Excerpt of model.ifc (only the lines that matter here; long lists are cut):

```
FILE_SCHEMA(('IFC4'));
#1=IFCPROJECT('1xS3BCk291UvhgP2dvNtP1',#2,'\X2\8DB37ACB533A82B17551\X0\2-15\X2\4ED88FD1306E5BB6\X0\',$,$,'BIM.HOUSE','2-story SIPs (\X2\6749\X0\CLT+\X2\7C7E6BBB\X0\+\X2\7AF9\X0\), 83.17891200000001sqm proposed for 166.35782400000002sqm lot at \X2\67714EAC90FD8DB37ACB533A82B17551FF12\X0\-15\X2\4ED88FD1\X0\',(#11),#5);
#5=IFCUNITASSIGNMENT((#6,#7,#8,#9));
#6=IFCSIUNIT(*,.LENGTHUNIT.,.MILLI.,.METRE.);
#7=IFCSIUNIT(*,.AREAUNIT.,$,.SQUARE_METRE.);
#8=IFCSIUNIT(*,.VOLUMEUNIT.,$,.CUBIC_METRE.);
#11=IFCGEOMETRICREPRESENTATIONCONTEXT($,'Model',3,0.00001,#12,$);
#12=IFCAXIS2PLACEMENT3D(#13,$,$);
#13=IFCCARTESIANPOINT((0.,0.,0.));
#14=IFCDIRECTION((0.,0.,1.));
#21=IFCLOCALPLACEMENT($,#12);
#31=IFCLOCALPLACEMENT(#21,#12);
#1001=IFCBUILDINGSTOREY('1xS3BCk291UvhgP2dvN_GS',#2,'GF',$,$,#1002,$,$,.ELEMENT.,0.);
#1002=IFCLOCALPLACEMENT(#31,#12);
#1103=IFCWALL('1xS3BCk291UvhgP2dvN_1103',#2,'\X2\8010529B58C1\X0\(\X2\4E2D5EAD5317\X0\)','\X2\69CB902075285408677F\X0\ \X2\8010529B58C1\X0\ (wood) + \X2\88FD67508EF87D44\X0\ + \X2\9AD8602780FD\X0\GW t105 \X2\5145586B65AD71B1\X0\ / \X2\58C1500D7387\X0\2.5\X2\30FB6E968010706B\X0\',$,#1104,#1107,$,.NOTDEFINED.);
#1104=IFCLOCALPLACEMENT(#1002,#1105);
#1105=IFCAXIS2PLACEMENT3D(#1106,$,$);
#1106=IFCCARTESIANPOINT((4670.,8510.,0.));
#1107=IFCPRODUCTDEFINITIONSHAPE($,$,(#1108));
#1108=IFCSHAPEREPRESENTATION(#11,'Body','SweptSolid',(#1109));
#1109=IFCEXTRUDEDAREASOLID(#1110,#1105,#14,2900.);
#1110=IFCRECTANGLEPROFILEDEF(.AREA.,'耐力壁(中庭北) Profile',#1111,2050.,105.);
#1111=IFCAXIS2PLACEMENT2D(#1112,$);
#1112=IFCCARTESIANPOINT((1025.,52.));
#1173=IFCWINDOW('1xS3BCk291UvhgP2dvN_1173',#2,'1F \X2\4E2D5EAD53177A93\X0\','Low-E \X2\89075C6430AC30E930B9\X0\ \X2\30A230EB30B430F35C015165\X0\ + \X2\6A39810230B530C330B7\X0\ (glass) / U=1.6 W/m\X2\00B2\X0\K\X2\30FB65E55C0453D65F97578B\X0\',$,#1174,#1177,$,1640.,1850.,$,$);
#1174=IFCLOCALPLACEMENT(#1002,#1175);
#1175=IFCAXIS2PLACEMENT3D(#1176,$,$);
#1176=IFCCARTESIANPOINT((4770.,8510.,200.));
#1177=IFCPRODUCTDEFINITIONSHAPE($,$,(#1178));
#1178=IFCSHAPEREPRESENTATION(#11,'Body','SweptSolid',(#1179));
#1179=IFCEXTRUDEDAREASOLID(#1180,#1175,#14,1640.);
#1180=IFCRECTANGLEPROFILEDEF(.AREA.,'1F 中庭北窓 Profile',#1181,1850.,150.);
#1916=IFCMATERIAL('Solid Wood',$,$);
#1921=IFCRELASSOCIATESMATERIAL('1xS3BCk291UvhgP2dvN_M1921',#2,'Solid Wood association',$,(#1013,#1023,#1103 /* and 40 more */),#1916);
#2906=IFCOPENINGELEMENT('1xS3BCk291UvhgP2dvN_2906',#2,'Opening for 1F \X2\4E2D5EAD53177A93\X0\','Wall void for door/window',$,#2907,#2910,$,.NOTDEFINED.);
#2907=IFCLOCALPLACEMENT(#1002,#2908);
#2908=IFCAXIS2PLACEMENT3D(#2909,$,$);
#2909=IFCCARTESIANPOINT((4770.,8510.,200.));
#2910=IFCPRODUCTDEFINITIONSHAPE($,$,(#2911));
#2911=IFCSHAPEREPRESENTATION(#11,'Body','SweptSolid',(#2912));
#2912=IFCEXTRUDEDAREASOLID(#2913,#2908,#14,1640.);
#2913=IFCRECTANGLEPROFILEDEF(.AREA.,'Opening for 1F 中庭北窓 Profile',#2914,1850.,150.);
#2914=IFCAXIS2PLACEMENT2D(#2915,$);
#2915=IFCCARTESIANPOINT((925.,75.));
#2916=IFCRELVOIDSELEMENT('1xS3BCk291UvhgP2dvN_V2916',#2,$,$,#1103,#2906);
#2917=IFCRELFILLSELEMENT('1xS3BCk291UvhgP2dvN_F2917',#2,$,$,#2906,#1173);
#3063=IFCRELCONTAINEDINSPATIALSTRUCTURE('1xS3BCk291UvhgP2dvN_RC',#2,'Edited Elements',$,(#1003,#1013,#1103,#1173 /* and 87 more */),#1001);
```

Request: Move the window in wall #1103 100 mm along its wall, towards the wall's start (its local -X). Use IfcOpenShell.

```python
import ifcopenshell
import ifcopenshell.api.geometry
import ifcopenshell.util.placement

model = ifcopenshell.open("model.ifc")

window = model.by_guid("1xS3BCk291UvhgP2dvN_1173")
opening = window.FillsVoids[0].RelatingOpeningElement
wall = opening.VoidsElements[0].RelatingBuildingElement

wall_matrix = ifcopenshell.util.placement.get_local_placement(wall.ObjectPlacement)
shift = wall_matrix[:3, 0] * -100.0
before = ifcopenshell.util.placement.get_local_placement(window.ObjectPlacement)[:3, 3].copy()

# The window is not placed relative to its opening, so move both.
for product in (opening, window):
    matrix = ifcopenshell.util.placement.get_local_placement(product.ObjectPlacement)
    matrix[:3, 3] += shift
    ifcopenshell.api.geometry.edit_object_placement(model, product=product, matrix=matrix, is_si=False)

after = ifcopenshell.util.placement.get_local_placement(window.ObjectPlacement)[:3, 3]
print("window moved by", (after - before).round(3) + 0.0)

model.write("model_v2.ifc")
```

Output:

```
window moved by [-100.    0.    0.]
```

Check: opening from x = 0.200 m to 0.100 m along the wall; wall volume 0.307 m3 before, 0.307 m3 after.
